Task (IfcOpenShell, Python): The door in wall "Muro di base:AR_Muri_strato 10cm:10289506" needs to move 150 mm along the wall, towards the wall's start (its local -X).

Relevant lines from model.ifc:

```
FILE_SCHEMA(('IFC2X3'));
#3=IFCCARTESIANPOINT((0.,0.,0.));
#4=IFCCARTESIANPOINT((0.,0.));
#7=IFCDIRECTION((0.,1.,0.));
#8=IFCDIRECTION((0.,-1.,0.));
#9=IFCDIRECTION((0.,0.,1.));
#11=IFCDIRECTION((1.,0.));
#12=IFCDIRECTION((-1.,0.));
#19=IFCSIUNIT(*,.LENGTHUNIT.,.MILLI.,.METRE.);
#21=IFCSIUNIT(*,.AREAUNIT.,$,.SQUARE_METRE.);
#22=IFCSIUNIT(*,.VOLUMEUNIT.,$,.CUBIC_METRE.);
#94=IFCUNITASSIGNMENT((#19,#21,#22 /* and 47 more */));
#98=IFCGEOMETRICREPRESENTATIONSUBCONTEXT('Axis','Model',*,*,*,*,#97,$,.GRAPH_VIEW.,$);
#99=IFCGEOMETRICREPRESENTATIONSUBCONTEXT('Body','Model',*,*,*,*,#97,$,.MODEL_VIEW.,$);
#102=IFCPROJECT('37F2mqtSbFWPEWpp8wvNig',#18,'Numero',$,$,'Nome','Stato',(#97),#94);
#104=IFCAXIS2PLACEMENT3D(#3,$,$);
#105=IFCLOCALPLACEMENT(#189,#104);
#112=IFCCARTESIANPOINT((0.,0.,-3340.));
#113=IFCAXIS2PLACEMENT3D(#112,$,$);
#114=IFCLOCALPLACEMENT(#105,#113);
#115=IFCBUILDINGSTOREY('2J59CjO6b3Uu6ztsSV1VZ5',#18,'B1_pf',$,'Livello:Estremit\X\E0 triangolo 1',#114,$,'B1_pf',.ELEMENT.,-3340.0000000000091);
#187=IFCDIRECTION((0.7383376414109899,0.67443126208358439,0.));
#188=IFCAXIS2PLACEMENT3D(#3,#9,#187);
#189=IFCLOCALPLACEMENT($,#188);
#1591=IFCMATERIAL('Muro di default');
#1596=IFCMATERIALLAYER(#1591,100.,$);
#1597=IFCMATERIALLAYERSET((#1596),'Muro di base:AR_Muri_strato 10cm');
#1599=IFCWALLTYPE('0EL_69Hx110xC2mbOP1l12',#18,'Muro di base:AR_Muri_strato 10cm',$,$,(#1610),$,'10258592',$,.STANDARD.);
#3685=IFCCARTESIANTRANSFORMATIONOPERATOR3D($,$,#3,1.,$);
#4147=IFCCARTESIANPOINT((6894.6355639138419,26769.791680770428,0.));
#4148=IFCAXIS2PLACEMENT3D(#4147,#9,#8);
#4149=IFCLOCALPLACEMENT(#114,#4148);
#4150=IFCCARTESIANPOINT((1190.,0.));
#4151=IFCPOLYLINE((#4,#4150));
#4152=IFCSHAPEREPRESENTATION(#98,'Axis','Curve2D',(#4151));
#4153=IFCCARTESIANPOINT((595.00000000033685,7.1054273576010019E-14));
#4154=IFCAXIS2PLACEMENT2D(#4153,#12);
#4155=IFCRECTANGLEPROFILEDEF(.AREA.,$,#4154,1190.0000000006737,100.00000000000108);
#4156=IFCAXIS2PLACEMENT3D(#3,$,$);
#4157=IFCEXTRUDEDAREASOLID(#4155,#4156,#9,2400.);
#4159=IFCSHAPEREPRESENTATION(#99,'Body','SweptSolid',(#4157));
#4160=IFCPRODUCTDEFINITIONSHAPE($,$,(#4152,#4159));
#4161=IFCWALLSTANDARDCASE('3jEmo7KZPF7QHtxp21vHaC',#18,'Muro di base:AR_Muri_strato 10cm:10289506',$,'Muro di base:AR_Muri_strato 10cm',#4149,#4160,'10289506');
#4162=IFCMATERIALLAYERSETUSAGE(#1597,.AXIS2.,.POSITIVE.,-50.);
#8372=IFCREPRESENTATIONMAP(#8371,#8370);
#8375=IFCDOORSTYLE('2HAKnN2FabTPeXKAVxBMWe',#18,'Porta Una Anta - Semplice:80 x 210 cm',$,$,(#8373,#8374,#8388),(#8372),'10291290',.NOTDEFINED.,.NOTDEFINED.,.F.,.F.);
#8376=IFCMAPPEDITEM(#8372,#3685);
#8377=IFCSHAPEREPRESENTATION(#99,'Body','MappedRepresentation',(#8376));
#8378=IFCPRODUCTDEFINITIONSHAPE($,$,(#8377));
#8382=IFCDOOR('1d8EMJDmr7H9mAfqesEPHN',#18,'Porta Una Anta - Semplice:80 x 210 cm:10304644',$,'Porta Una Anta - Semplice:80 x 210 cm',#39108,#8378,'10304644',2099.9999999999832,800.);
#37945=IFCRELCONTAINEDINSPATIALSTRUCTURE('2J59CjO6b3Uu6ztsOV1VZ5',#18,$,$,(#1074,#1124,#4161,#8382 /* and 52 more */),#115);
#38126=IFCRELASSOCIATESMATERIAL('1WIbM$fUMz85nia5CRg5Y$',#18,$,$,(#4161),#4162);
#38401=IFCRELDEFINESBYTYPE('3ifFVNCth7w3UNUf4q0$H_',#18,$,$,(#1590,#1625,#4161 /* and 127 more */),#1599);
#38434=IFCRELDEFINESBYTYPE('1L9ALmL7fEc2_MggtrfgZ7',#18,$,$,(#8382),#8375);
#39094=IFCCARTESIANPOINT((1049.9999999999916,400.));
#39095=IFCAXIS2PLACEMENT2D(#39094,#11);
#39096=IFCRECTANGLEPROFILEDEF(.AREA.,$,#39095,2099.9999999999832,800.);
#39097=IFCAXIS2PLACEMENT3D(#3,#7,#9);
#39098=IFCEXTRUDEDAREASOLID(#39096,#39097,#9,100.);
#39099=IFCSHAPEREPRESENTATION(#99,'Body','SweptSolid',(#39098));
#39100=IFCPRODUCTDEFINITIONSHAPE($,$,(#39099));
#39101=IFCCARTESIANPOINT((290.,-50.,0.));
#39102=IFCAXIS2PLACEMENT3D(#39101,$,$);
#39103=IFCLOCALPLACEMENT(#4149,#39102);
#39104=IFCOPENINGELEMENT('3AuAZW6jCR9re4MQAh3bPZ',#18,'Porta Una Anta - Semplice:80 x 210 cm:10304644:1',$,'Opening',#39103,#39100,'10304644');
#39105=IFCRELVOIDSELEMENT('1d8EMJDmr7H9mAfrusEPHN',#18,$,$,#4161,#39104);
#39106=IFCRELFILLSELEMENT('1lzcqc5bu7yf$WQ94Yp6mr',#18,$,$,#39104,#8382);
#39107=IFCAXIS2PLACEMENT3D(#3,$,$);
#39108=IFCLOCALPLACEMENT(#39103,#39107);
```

```python
import ifcopenshell
import ifcopenshell.api.geometry
import ifcopenshell.util.placement

model = ifcopenshell.open("model.ifc")

door = model.by_guid("1d8EMJDmr7H9mAfqesEPHN")
opening = door.FillsVoids[0].RelatingOpeningElement
wall = opening.VoidsElements[0].RelatingBuildingElement

wall_matrix = ifcopenshell.util.placement.get_local_placement(wall.ObjectPlacement)
shift = wall_matrix[:3, 0] * -150.0
before = ifcopenshell.util.placement.get_local_placement(door.ObjectPlacement)[:3, 3].copy()

# The door is placed relative to its opening, so it follows when the opening moves.
matrix = ifcopenshell.util.placement.get_local_placement(opening.ObjectPlacement)
matrix[:3, 3] += shift
ifcopenshell.api.geometry.edit_object_placement(
    model, product=opening, matrix=matrix, is_si=False, should_transform_children=True
)

after = ifcopenshell.util.placement.get_local_placement(door.ObjectPlacement)[:3, 3]
print("door moved by", (after - before).round(3) + 0.0)

model.write("model_updated.ifc")
```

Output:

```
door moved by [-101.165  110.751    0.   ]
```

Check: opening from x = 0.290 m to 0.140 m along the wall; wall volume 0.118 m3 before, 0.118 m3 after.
